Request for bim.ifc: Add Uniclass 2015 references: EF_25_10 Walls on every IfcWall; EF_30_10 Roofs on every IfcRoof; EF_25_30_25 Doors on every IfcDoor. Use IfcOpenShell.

First a look at what the model holds.

```python
import ifcopenshell

model = ifcopenshell.open("bim.ifc")
print(model.schema)
print("classifications:", [c.Name for c in model.by_type("IfcClassification")])
for ifc_class in ("IfcDoor", "IfcRoof", "IfcStair", "IfcWall", "IfcWindow"):
    print(ifc_class, len(model.by_type(ifc_class)))
```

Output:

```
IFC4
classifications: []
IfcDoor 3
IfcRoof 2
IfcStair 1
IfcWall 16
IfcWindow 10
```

```python
import ifcopenshell
import ifcopenshell.api.classification

model = ifcopenshell.open("bim.ifc")

system = ifcopenshell.api.classification.add_classification(model, classification="Uniclass 2015")

codes = {
    "IfcWall": ("EF_25_10", "Walls"),
    "IfcRoof": ("EF_30_10", "Roofs"),
    "IfcDoor": ("EF_25_30_25", "Doors"),
}
for ifc_class, (code, name) in codes.items():
    products = model.by_type(ifc_class)
    ifcopenshell.api.classification.add_reference(
        model, products=products, classification=system, identification=code, name=name
    )
    print(code, len(products))

model.write("bim_rev.ifc")
```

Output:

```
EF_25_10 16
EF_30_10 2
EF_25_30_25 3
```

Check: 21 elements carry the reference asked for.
